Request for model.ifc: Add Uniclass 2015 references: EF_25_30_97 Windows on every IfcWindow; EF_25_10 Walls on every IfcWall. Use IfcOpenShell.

First a look at what the model holds.

```python
import ifcopenshell

model = ifcopenshell.open("model.ifc")
print(model.schema)
print("classifications:", [c.Name for c in model.by_type("IfcClassification")])
for ifc_class in ("IfcDoor", "IfcRoof", "IfcStair", "IfcWall", "IfcWindow"):
    print(ifc_class, len(model.by_type(ifc_class)))
```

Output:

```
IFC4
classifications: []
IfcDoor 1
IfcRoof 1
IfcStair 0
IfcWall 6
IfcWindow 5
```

```python
import ifcopenshell
import ifcopenshell.api.classification

model = ifcopenshell.open("model.ifc")

system = ifcopenshell.api.classification.add_classification(model, classification="Uniclass 2015")

codes = {
    "IfcWindow": ("EF_25_30_97", "Windows"),
    "IfcWall": ("EF_25_10", "Walls"),
}
for ifc_class, (code, name) in codes.items():
    products = model.by_type(ifc_class)
    ifcopenshell.api.classification.add_reference(
        model, products=products, classification=system, identification=code, name=name
    )
    print(code, len(products))

model.write("model_edited.ifc")
```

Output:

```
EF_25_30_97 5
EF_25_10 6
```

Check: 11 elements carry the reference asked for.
